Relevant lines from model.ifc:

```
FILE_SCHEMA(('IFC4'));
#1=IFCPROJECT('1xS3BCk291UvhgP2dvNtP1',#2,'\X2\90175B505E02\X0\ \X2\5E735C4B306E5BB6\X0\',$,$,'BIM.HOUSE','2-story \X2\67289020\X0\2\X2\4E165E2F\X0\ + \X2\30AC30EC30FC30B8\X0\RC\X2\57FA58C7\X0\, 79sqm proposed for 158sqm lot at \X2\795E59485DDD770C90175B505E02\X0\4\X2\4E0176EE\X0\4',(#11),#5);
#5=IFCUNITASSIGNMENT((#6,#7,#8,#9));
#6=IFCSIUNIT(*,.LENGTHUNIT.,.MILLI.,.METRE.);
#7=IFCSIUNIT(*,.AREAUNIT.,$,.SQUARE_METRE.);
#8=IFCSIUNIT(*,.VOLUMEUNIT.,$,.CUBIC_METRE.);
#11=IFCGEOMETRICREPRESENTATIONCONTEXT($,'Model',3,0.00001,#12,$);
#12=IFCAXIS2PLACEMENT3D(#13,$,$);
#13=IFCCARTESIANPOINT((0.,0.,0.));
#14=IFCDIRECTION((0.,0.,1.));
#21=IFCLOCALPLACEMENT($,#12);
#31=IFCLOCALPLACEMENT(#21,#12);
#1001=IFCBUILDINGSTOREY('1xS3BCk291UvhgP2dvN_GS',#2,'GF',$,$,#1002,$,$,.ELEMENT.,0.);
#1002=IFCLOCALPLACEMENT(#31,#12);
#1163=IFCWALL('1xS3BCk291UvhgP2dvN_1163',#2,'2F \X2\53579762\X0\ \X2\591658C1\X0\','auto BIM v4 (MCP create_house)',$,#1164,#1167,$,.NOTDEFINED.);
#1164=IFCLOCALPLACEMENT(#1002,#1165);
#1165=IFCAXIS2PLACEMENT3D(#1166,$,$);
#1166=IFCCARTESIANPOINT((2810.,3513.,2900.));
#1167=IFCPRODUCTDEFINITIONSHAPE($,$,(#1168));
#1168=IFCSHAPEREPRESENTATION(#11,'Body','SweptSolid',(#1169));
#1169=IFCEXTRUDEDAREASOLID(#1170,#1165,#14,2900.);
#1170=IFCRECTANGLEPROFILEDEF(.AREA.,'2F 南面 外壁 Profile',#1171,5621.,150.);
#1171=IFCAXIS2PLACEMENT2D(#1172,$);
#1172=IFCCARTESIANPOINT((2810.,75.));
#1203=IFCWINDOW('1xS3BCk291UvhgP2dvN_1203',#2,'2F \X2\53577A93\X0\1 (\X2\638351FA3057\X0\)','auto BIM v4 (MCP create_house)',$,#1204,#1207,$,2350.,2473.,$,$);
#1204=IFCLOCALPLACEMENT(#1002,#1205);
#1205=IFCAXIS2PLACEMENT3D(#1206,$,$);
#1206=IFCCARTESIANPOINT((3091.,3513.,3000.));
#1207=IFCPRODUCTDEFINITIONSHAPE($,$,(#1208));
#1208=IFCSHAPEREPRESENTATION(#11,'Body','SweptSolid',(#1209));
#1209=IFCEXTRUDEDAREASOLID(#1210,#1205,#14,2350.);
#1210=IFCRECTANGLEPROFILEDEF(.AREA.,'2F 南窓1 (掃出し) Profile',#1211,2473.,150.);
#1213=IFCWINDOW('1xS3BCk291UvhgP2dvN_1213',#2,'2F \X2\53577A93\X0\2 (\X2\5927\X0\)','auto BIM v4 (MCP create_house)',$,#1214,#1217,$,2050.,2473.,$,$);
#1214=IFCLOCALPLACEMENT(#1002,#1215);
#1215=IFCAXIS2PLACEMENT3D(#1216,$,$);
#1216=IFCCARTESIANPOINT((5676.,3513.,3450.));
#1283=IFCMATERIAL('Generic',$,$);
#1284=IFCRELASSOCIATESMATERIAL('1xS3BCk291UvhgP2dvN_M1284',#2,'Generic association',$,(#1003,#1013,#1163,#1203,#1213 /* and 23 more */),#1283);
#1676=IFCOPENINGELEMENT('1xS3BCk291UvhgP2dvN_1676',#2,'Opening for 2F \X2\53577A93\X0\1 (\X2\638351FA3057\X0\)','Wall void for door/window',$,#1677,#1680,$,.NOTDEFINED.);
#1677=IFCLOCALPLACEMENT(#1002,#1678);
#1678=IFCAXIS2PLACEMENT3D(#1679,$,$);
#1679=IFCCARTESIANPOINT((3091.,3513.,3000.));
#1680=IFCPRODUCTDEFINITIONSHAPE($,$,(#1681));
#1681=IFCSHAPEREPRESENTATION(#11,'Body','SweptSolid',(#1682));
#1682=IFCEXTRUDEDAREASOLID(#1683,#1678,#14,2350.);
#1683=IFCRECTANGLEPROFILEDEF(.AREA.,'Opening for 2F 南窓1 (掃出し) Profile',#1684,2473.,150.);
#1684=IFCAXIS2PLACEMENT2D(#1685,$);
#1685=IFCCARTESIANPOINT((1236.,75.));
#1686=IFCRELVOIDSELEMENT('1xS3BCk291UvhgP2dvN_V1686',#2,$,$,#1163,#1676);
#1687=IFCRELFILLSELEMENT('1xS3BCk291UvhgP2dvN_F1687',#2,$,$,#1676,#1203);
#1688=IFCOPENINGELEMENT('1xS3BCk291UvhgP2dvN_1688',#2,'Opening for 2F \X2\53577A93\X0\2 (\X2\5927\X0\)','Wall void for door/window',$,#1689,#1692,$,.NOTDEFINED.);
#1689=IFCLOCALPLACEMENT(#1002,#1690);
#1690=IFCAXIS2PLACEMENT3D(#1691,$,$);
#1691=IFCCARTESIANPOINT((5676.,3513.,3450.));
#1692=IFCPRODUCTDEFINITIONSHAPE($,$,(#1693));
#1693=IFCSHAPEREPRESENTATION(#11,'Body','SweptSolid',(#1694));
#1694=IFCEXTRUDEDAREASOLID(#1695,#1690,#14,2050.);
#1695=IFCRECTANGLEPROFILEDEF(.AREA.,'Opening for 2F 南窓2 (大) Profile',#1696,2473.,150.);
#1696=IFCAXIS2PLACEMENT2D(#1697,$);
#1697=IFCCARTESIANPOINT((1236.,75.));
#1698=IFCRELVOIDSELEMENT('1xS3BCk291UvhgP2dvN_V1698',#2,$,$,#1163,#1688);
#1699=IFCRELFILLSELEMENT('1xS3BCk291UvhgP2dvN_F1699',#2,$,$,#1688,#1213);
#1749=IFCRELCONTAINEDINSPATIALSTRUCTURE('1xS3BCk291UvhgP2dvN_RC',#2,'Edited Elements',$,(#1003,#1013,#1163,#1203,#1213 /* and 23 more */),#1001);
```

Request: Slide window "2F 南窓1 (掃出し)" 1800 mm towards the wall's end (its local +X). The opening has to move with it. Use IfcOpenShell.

```python
import ifcopenshell
import ifcopenshell.api.geometry
import ifcopenshell.util.placement
import ifcopenshell.util.unit

model = ifcopenshell.open("model.ifc")
unit_scale = ifcopenshell.util.unit.calculate_unit_scale(model)

window = model.by_guid("1xS3BCk291UvhgP2dvN_1203")
opening = window.FillsVoids[0].RelatingOpeningElement
wall = opening.VoidsElements[0].RelatingBuildingElement

wall_matrix = ifcopenshell.util.placement.get_local_placement(wall.ObjectPlacement)
shift = wall_matrix[:3, 0] * 1.8 / unit_scale
before = ifcopenshell.util.placement.get_local_placement(window.ObjectPlacement)[:3, 3].copy()

# The window is not placed relative to its opening, so move both.
for product in (opening, window):
    matrix = ifcopenshell.util.placement.get_local_placement(product.ObjectPlacement)
    matrix[:3, 3] += shift
    ifcopenshell.api.geometry.edit_object_placement(model, product=product, matrix=matrix, is_si=False)

after = ifcopenshell.util.placement.get_local_placement(window.ObjectPlacement)[:3, 3]
print("window moved by", (after - before).round(3) + 0.0)

model.write("model-out.ifc")
```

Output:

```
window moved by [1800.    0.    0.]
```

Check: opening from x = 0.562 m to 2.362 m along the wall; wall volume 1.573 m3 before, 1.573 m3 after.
